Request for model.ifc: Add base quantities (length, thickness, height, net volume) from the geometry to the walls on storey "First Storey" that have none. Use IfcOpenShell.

First a look at what the model holds.

```python
import ifcopenshell
import ifcopenshell.util.element
import ifcopenshell.util.unit

model = ifcopenshell.open("model.ifc")
print(model.schema)
for unit_type in ("LENGTHUNIT", "AREAUNIT", "VOLUMEUNIT"):
    print(unit_type, ifcopenshell.util.unit.calculate_unit_scale(model, unit_type))
storey = next(s for s in model.by_type("IfcBuildingStorey") if s.Name == "First Storey")
walls = [e for e in ifcopenshell.util.element.get_decomposition(storey) if e.is_a("IfcWall")]
for e in sorted(walls, key=lambda e: e.id()):
    print(e.id(), e.is_a(), e.Name, list(ifcopenshell.util.element.get_psets(e, qtos_only=True)), sep=" | ")
```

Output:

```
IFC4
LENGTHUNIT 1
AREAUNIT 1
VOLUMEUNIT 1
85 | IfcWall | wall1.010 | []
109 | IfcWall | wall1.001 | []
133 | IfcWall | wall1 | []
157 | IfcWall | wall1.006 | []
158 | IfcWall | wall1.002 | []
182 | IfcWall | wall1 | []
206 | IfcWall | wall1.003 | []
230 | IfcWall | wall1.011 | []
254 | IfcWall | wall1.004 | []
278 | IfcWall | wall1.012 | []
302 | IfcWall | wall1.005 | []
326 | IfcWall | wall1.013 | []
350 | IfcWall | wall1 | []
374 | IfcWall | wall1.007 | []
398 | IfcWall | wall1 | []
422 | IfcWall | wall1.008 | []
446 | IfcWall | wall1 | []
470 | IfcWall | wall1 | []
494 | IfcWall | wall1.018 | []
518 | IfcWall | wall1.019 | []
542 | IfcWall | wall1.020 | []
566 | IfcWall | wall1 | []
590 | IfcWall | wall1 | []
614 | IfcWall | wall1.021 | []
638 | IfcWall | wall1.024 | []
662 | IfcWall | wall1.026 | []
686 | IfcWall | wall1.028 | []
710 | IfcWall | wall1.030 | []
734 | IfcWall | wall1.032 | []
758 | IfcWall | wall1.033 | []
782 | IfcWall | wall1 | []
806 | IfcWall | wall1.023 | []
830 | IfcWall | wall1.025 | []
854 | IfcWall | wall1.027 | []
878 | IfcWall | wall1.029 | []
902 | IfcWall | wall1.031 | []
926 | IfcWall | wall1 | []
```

```python
import ifcopenshell
import ifcopenshell.api.pset
import ifcopenshell.geom
import ifcopenshell.util.element
import ifcopenshell.util.shape
import ifcopenshell.util.unit

model = ifcopenshell.open("model.ifc")
unit_scale = ifcopenshell.util.unit.calculate_unit_scale(model)
volume_scale = ifcopenshell.util.unit.calculate_unit_scale(model, "VOLUMEUNIT")
settings = ifcopenshell.geom.settings()

storey = next(s for s in model.by_type("IfcBuildingStorey") if s.Name == "First Storey")
walls = [e for e in ifcopenshell.util.element.get_decomposition(storey) if e.is_a("IfcWall")]

for e in sorted(walls, key=lambda e: e.id()):
    if ifcopenshell.util.element.get_psets(e, qtos_only=True, should_inherit=False):
        continue
    # Geometry comes back in metres, in the element's own axes.
    shape = ifcopenshell.geom.create_shape(settings, e)
    values = {
        "Length": ifcopenshell.util.shape.get_x(shape.geometry) / unit_scale,
        "Width": ifcopenshell.util.shape.get_y(shape.geometry) / unit_scale,
        "Height": ifcopenshell.util.shape.get_z(shape.geometry) / unit_scale,
        "NetVolume": ifcopenshell.util.shape.get_volume(shape.geometry) / volume_scale,
    }
    qto = ifcopenshell.api.pset.add_qto(model, product=e, name="Qto_WallBaseQuantities")
    ifcopenshell.api.pset.edit_qto(model, qto=qto, properties=values)
    print(e.id(), {k: round(v, 3) for k, v in values.items()})

model.write("model_rev.ifc")
```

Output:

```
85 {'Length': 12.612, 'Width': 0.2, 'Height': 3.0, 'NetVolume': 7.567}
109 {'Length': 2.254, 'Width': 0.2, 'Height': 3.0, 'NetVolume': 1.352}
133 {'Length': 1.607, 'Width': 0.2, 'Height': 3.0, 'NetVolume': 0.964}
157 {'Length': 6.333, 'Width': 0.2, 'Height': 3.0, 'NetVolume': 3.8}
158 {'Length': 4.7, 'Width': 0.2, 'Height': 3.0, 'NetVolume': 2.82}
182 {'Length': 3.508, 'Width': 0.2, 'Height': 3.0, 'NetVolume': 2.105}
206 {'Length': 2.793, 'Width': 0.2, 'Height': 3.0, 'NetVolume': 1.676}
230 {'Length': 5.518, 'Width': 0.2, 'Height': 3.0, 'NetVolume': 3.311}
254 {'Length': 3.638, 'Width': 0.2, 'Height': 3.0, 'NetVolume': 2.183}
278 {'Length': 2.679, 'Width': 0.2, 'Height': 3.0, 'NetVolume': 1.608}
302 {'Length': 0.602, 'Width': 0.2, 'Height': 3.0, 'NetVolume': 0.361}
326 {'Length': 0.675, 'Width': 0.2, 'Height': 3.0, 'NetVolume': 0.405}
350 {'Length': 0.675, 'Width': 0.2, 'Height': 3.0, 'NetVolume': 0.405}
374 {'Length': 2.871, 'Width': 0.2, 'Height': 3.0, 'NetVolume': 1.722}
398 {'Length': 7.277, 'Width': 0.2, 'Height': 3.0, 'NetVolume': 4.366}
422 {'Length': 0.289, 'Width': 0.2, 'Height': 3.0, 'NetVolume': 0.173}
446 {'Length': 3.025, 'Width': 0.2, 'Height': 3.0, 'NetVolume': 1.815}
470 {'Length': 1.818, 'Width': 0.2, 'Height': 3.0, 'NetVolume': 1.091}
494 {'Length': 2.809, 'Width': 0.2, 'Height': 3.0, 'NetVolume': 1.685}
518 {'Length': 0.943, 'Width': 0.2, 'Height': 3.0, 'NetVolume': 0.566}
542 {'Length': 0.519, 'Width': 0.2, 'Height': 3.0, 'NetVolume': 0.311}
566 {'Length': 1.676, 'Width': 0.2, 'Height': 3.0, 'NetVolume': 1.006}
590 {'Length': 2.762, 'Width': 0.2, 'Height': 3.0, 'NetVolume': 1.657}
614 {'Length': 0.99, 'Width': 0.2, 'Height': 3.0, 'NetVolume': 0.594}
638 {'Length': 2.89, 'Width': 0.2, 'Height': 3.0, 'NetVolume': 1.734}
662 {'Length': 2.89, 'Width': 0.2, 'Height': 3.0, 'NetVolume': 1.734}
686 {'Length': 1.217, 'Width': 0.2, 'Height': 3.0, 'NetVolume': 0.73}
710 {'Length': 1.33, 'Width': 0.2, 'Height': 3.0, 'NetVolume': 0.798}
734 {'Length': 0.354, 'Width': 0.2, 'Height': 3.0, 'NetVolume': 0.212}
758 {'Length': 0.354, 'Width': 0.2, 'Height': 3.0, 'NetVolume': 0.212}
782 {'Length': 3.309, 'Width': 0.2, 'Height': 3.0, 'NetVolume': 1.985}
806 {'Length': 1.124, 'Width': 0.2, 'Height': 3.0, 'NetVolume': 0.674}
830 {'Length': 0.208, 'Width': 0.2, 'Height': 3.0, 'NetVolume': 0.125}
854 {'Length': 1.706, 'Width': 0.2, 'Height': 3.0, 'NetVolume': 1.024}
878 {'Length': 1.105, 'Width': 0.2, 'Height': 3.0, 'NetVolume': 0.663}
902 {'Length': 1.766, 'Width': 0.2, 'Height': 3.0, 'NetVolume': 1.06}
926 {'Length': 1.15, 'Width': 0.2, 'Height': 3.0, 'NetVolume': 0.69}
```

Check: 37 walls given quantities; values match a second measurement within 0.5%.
